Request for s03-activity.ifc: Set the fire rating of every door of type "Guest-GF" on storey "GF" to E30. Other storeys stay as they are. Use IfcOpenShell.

First a look at what the model holds.

```python
import ifcopenshell
import ifcopenshell.util.element

model = ifcopenshell.open("s03-activity.ifc")
print(model.schema)
storey = next(s for s in model.by_type("IfcBuildingStorey") if s.Name == "GF")
doors = [e for e in ifcopenshell.util.element.get_decomposition(storey) if e.is_a("IfcDoor")]
seen = {}
for e in doors:
    element_type = ifcopenshell.util.element.get_type(e)
    key = (element_type.Name if element_type != e and element_type else None, ifcopenshell.util.element.get_pset(e, "Pset_DoorCommon", "FireRating"))
    seen[key] = seen.get(key, 0) + 1
for (name, value), count in sorted(seen.items(), key=str):
    print(count, "x", name, "|", value)
```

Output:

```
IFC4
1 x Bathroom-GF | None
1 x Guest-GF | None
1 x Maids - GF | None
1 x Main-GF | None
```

```python
import ifcopenshell
import ifcopenshell.api.pset
import ifcopenshell.util.element

model = ifcopenshell.open("s03-activity.ifc")

storey = next(s for s in model.by_type("IfcBuildingStorey") if s.Name == "GF")
doors = [e for e in ifcopenshell.util.element.get_decomposition(storey) if e.is_a("IfcDoor")]

count = 0
for e in doors:
    element_type = ifcopenshell.util.element.get_type(e)
    if element_type in (None, e) or element_type.Name != "Guest-GF":
        continue
    # add_pset returns the element's existing set when there is one.
    pset = ifcopenshell.api.pset.add_pset(model, product=e, name="Pset_DoorCommon")
    ifcopenshell.api.pset.edit_pset(model, pset=pset, properties={"FireRating": "E30"})
    count += 1

print(count, "doors updated")

model.write("s03-activity_edited.ifc")
```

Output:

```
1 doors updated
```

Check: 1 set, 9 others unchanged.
